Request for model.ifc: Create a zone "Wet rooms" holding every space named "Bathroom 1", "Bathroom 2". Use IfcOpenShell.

First a look at what the model holds.

```python
import ifcopenshell

model = ifcopenshell.open("model.ifc")
print(model.schema)
seen = {}
for space in model.by_type("IfcSpace"):
    seen[space.LongName] = seen.get(space.LongName, 0) + 1
for name, count in sorted(seen.items(), key=str):
    print(count, "x", name)
print("zones:", [z.Name for z in model.by_type("IfcZone")][:20])
```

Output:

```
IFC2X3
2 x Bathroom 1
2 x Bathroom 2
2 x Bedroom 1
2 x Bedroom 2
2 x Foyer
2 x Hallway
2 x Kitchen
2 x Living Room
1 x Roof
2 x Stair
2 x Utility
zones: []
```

```python
import ifcopenshell
import ifcopenshell.api.group
import ifcopenshell.api.root

model = ifcopenshell.open("model.ifc")

names = {"Bathroom 1", "Bathroom 2"}
spaces = [s for s in model.by_type("IfcSpace") if s.LongName in names]

zone = ifcopenshell.api.root.create_entity(model, ifc_class="IfcZone", name="Wet rooms")
ifcopenshell.api.group.assign_group(model, products=spaces, group=zone)
print(len(spaces), "spaces in", zone.Name)

model.write("model_updated.ifc")
```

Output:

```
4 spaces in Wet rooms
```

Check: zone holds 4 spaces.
